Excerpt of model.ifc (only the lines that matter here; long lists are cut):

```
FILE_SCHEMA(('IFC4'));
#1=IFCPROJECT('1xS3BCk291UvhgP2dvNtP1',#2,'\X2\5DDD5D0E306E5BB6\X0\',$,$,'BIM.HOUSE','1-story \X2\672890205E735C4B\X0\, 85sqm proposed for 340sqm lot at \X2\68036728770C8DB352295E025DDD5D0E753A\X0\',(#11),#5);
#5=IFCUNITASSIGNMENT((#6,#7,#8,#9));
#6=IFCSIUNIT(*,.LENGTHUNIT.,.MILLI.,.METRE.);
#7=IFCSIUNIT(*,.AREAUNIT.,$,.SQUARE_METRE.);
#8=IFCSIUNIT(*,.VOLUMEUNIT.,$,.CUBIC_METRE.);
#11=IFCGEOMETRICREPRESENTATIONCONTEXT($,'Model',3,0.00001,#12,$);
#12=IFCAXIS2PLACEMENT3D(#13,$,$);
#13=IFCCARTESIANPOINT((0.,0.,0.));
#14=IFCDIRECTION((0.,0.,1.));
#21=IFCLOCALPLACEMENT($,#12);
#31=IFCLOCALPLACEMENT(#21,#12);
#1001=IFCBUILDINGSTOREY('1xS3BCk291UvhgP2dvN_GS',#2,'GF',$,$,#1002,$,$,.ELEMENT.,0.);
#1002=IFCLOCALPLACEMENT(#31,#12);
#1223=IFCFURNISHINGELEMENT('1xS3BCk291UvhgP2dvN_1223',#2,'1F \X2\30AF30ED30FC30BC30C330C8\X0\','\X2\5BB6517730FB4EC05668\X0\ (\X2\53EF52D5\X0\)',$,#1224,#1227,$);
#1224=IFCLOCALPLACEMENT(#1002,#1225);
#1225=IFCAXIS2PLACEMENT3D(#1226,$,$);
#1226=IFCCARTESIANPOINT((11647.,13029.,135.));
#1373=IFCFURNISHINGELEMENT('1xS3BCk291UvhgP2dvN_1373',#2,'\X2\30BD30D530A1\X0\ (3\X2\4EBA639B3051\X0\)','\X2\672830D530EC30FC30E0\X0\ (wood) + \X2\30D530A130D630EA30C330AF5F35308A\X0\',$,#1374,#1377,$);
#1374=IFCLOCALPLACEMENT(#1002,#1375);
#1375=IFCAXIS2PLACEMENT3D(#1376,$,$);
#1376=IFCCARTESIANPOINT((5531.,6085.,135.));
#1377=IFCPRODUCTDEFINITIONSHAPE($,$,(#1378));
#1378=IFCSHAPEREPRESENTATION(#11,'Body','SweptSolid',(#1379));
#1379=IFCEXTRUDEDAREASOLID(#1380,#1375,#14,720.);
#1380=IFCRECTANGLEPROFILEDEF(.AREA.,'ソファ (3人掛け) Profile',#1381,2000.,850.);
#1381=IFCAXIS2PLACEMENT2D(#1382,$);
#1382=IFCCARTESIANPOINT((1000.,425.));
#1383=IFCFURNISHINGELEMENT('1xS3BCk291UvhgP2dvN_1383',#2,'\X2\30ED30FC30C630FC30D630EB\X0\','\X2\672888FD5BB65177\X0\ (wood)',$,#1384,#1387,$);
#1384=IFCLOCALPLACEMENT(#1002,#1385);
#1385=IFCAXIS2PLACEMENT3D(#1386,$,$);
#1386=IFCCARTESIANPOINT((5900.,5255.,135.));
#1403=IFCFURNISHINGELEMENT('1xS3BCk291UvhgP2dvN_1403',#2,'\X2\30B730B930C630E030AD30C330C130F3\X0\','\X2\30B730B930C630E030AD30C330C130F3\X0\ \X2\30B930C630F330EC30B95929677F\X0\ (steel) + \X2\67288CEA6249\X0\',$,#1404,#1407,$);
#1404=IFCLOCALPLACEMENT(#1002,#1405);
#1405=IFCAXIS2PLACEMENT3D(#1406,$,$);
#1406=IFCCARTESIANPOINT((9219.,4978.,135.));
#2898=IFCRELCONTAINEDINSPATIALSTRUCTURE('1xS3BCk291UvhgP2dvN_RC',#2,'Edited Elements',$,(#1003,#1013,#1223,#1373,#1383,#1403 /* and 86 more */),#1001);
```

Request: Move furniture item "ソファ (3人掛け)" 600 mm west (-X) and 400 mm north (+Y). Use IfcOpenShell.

```python
import ifcopenshell
import ifcopenshell.api.geometry
import ifcopenshell.util.placement

model = ifcopenshell.open("model.ifc")

item = model.by_guid("1xS3BCk291UvhgP2dvN_1373")
matrix = ifcopenshell.util.placement.get_local_placement(item.ObjectPlacement)
matrix[0, 3] -= 600.0
matrix[1, 3] += 400.0
ifcopenshell.api.geometry.edit_object_placement(model, product=item, matrix=matrix, is_si=False)

print(ifcopenshell.util.placement.get_local_placement(item.ObjectPlacement).round(3) + 0.0)

model.write("model_v2.ifc")
```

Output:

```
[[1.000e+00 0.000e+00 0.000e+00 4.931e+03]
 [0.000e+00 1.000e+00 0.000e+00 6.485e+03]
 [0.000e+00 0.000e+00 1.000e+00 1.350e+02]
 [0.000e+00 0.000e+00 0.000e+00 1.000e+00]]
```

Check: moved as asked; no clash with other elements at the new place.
